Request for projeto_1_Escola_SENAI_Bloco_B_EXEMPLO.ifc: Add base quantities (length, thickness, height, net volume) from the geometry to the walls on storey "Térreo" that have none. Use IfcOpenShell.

First a look at what the model holds.

```python
import ifcopenshell
import ifcopenshell.util.element
import ifcopenshell.util.unit

model = ifcopenshell.open("projeto_1_Escola_SENAI_Bloco_B_EXEMPLO.ifc")
print(model.schema)
for unit_type in ("LENGTHUNIT", "AREAUNIT", "VOLUMEUNIT"):
    print(unit_type, ifcopenshell.util.unit.calculate_unit_scale(model, unit_type))
storey = next(s for s in model.by_type("IfcBuildingStorey") if s.Name == "Térreo")
walls = [e for e in ifcopenshell.util.element.get_decomposition(storey) if e.is_a("IfcWall")]
for e in sorted(walls, key=lambda e: e.id()):
    print(e.id(), e.is_a(), e.Name, list(ifcopenshell.util.element.get_psets(e, qtos_only=True)), sep=" | ")
```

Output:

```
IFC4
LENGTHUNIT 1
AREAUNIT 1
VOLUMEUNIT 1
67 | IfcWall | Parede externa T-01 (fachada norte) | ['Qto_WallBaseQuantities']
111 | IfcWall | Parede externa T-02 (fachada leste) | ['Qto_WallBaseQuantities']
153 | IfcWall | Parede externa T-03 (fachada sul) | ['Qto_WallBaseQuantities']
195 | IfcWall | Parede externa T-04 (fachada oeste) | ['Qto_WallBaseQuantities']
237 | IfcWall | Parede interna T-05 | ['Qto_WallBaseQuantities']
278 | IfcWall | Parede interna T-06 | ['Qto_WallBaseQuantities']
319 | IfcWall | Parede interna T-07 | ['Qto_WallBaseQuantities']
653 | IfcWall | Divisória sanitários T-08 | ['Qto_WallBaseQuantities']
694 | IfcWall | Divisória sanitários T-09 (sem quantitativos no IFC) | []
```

```python
import ifcopenshell
import ifcopenshell.api.pset
import ifcopenshell.geom
import ifcopenshell.util.element
import ifcopenshell.util.shape
import ifcopenshell.util.unit

model = ifcopenshell.open("projeto_1_Escola_SENAI_Bloco_B_EXEMPLO.ifc")
unit_scale = ifcopenshell.util.unit.calculate_unit_scale(model)
volume_scale = ifcopenshell.util.unit.calculate_unit_scale(model, "VOLUMEUNIT")
settings = ifcopenshell.geom.settings()

storey = next(s for s in model.by_type("IfcBuildingStorey") if s.Name == "Térreo")
walls = [e for e in ifcopenshell.util.element.get_decomposition(storey) if e.is_a("IfcWall")]

for e in sorted(walls, key=lambda e: e.id()):
    if ifcopenshell.util.element.get_psets(e, qtos_only=True, should_inherit=False):
        continue
    # Geometry comes back in metres, in the element's own axes.
    shape = ifcopenshell.geom.create_shape(settings, e)
    values = {
        "Length": ifcopenshell.util.shape.get_x(shape.geometry) / unit_scale,
        "Width": ifcopenshell.util.shape.get_y(shape.geometry) / unit_scale,
        "Height": ifcopenshell.util.shape.get_z(shape.geometry) / unit_scale,
        "NetVolume": ifcopenshell.util.shape.get_volume(shape.geometry) / volume_scale,
    }
    qto = ifcopenshell.api.pset.add_qto(model, product=e, name="Qto_WallBaseQuantities")
    ifcopenshell.api.pset.edit_qto(model, qto=qto, properties=values)
    print(e.id(), {k: round(v, 3) for k, v in values.items()})

model.write("projeto_1_Escola_SENAI_Bloco_B_EXEMPLO-out.ifc")
```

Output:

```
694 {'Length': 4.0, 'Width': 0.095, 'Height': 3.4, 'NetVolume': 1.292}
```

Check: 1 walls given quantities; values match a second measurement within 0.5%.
